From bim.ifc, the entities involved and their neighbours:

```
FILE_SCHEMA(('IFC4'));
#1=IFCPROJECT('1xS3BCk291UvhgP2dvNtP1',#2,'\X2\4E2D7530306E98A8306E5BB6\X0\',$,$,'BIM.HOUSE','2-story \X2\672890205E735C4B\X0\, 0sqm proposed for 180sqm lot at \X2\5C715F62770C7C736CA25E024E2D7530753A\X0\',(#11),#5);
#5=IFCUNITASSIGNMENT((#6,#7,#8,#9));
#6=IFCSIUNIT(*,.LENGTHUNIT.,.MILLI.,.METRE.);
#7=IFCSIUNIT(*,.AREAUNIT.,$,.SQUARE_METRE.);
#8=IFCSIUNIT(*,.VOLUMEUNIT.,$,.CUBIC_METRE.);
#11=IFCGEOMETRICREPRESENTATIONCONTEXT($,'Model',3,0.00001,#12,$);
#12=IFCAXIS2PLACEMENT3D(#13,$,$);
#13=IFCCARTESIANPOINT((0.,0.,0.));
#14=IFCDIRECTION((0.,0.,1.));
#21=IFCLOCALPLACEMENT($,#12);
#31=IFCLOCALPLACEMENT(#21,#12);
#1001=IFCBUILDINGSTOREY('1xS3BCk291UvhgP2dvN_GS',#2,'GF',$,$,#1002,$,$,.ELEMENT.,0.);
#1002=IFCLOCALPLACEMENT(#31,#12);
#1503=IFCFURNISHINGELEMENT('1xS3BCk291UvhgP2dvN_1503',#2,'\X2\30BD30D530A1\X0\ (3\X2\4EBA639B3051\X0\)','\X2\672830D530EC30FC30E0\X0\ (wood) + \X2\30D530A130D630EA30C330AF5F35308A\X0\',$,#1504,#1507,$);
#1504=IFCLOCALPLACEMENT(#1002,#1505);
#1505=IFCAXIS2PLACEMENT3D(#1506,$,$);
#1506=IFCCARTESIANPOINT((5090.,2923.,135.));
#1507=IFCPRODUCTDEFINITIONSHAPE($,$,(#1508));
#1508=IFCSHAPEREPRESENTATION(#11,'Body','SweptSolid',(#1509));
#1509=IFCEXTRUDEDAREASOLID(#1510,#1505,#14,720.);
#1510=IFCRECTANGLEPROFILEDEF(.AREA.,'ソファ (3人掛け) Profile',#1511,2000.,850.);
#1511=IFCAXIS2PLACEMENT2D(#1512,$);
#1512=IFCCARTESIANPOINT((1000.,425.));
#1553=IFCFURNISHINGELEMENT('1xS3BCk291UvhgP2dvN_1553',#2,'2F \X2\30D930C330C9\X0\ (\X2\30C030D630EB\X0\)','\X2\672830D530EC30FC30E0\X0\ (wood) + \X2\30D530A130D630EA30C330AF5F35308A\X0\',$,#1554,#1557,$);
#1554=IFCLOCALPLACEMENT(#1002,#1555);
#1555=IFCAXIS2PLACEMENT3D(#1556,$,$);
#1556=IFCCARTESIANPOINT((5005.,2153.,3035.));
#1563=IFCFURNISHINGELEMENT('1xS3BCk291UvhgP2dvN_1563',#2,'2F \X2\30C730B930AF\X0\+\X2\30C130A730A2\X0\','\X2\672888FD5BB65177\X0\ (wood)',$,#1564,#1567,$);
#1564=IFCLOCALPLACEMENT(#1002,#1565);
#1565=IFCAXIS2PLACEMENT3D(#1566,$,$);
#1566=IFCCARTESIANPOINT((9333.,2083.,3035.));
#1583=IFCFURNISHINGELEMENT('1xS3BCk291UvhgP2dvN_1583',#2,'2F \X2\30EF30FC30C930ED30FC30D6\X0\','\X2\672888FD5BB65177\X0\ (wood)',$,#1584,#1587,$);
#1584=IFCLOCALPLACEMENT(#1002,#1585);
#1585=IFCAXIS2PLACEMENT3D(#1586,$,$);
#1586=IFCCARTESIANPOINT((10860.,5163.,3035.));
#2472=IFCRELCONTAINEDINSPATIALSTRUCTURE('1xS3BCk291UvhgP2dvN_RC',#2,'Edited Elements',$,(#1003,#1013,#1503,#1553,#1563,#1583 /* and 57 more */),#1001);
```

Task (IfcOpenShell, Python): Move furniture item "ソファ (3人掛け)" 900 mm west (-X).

```python
import ifcopenshell
import ifcopenshell.api.geometry
import ifcopenshell.util.placement
import ifcopenshell.util.unit

model = ifcopenshell.open("bim.ifc")
unit_scale = ifcopenshell.util.unit.calculate_unit_scale(model)

item = model.by_guid("1xS3BCk291UvhgP2dvN_1503")
matrix = ifcopenshell.util.placement.get_local_placement(item.ObjectPlacement)
matrix[0, 3] -= 0.9 / unit_scale
ifcopenshell.api.geometry.edit_object_placement(model, product=item, matrix=matrix, is_si=False)

print(ifcopenshell.util.placement.get_local_placement(item.ObjectPlacement).round(3) + 0.0)

model.write("bim_rev.ifc")
```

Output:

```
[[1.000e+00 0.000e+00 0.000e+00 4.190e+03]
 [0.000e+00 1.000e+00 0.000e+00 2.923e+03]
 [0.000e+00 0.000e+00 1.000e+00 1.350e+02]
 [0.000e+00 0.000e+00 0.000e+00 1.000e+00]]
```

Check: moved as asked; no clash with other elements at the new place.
